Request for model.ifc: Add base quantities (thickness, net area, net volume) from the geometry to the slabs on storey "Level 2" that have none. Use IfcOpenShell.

First a look at what the model holds.

```python
import ifcopenshell
import ifcopenshell.util.element
import ifcopenshell.util.unit

model = ifcopenshell.open("model.ifc")
print(model.schema)
for unit_type in ("LENGTHUNIT", "AREAUNIT", "VOLUMEUNIT"):
    print(unit_type, ifcopenshell.util.unit.calculate_unit_scale(model, unit_type))
storey = next(s for s in model.by_type("IfcBuildingStorey") if s.Name == "Level 2")
slabs = [e for e in ifcopenshell.util.element.get_decomposition(storey) if e.is_a("IfcSlab")]
for e in sorted(slabs, key=lambda e: e.id()):
    print(e.id(), e.is_a(), e.Name, list(ifcopenshell.util.element.get_psets(e, qtos_only=True)), sep=" | ")
```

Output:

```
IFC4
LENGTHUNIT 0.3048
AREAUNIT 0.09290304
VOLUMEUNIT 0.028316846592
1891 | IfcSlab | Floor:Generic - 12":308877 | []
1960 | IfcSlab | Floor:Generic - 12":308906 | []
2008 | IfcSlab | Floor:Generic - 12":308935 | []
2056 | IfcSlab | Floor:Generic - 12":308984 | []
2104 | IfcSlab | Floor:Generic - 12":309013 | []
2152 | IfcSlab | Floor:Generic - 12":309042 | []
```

```python
import ifcopenshell
import ifcopenshell.api.pset
import ifcopenshell.geom
import ifcopenshell.util.element
import ifcopenshell.util.shape
import ifcopenshell.util.unit

model = ifcopenshell.open("model.ifc")
unit_scale = ifcopenshell.util.unit.calculate_unit_scale(model)
area_scale = ifcopenshell.util.unit.calculate_unit_scale(model, "AREAUNIT")
volume_scale = ifcopenshell.util.unit.calculate_unit_scale(model, "VOLUMEUNIT")
settings = ifcopenshell.geom.settings()

storey = next(s for s in model.by_type("IfcBuildingStorey") if s.Name == "Level 2")
slabs = [e for e in ifcopenshell.util.element.get_decomposition(storey) if e.is_a("IfcSlab")]

for e in sorted(slabs, key=lambda e: e.id()):
    if ifcopenshell.util.element.get_psets(e, qtos_only=True, should_inherit=False):
        continue
    # Geometry comes back in metres, in the element's own axes.
    shape = ifcopenshell.geom.create_shape(settings, e)
    values = {
        "Width": ifcopenshell.util.shape.get_z(shape.geometry) / unit_scale,
        "NetArea": ifcopenshell.util.shape.get_footprint_area(shape.geometry) / area_scale,
        "NetVolume": ifcopenshell.util.shape.get_volume(shape.geometry) / volume_scale,
    }
    qto = ifcopenshell.api.pset.add_qto(model, product=e, name="Qto_SlabBaseQuantities")
    ifcopenshell.api.pset.edit_qto(model, qto=qto, properties=values)
    print(e.id(), {k: round(v, 3) for k, v in values.items()})

model.write("model_rev.ifc")
```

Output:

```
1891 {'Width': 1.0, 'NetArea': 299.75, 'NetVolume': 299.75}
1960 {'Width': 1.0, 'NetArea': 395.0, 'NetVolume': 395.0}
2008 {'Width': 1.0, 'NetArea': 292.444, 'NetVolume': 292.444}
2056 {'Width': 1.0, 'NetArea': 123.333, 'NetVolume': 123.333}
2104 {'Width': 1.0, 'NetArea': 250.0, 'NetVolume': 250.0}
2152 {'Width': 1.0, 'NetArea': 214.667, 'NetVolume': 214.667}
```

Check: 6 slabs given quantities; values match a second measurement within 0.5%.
